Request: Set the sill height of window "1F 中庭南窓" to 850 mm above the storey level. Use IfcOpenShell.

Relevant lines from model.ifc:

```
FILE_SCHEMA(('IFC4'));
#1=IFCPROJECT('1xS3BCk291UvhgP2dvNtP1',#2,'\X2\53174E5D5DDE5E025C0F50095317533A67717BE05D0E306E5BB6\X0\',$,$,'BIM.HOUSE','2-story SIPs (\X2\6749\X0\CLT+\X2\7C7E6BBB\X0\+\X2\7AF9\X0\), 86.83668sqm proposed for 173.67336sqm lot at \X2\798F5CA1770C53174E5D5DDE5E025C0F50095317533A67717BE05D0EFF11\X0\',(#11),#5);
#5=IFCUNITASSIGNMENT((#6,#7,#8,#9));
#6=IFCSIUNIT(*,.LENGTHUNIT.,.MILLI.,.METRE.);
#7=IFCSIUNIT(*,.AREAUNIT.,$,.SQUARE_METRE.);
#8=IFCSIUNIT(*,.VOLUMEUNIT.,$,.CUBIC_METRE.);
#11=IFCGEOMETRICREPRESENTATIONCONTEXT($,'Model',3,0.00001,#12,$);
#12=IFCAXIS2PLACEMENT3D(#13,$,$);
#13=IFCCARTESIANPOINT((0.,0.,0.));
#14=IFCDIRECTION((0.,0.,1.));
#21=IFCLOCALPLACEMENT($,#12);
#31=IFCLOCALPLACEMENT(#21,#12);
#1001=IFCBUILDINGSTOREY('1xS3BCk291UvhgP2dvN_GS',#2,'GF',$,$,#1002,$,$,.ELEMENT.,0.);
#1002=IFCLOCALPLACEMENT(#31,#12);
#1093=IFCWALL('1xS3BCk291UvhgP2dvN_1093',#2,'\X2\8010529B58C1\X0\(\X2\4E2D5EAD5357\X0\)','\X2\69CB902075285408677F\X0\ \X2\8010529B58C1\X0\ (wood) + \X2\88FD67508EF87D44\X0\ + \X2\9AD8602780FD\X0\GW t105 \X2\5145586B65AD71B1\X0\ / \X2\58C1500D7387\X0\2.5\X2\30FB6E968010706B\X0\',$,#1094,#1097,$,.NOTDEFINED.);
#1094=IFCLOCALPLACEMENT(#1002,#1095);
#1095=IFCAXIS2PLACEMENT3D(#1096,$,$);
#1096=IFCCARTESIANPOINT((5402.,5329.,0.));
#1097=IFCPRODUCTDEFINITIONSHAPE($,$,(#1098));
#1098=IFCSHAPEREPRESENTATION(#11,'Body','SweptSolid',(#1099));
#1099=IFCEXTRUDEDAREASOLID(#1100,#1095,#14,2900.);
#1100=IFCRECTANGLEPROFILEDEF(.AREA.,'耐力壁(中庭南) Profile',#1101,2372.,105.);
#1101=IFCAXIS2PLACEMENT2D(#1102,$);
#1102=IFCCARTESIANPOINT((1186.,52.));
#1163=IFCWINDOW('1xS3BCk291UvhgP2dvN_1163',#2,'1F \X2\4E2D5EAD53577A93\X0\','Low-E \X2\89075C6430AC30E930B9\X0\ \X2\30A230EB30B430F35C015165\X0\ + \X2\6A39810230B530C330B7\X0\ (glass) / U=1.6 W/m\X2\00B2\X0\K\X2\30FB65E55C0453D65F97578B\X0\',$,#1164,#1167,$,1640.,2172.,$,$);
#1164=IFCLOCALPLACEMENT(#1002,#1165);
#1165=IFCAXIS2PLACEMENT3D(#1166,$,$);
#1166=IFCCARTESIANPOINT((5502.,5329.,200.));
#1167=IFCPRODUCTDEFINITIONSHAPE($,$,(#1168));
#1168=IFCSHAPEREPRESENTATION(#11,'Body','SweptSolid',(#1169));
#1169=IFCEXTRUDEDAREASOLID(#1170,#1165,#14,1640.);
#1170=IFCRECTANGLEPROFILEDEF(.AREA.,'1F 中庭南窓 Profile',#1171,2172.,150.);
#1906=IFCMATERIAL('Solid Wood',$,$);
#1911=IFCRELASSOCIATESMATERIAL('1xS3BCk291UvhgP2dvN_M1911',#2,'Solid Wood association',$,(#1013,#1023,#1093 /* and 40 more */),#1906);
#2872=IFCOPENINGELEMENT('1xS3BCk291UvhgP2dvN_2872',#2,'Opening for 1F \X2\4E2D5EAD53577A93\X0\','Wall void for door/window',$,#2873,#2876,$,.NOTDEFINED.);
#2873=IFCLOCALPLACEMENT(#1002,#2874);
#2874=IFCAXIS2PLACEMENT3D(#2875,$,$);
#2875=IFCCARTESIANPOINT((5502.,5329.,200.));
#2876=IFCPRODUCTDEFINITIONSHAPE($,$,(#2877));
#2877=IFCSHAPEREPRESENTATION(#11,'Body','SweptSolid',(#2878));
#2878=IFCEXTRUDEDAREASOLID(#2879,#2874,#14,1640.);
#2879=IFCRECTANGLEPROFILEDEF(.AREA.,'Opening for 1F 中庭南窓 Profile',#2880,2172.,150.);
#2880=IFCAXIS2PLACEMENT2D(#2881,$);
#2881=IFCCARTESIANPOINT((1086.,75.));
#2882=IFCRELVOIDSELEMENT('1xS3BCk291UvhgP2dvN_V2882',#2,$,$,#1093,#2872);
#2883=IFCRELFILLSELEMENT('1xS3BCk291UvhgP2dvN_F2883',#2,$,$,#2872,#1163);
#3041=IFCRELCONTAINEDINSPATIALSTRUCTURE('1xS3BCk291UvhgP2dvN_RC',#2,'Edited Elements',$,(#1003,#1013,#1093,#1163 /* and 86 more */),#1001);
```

```python
import numpy as np
import ifcopenshell
import ifcopenshell.api.geometry
import ifcopenshell.geom
import ifcopenshell.util.element
import ifcopenshell.util.placement
import ifcopenshell.util.shape
import ifcopenshell.util.unit

model = ifcopenshell.open("model.ifc")
unit_scale = ifcopenshell.util.unit.calculate_unit_scale(model)

window = model.by_id(1163)
opening = window.FillsVoids[0].RelatingOpeningElement
storey = ifcopenshell.util.element.get_container(window, ifc_class="IfcBuildingStorey")
level = ifcopenshell.util.placement.get_local_placement(storey.ObjectPlacement)[2, 3]

# The opening's origin need not be at the sill, so measure its lowest point.
shape = ifcopenshell.geom.create_shape(ifcopenshell.geom.settings(), opening)
bottom = ifcopenshell.util.shape.get_shape_bottom_elevation(shape, shape.geometry) / unit_scale
dz = level + 850.0 - bottom

shift = np.array([0.0, 0.0, dz])
# The window is not placed relative to its opening, so move both.
for product in (opening, window):
    matrix = ifcopenshell.util.placement.get_local_placement(product.ObjectPlacement)
    matrix[:3, 3] += shift
    ifcopenshell.api.geometry.edit_object_placement(model, product=product, matrix=matrix, is_si=False)

print(f"moved by {dz * unit_scale:+.3f} m")

model.write("model_updated.ifc")
```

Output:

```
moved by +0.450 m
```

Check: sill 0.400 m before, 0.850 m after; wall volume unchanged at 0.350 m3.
